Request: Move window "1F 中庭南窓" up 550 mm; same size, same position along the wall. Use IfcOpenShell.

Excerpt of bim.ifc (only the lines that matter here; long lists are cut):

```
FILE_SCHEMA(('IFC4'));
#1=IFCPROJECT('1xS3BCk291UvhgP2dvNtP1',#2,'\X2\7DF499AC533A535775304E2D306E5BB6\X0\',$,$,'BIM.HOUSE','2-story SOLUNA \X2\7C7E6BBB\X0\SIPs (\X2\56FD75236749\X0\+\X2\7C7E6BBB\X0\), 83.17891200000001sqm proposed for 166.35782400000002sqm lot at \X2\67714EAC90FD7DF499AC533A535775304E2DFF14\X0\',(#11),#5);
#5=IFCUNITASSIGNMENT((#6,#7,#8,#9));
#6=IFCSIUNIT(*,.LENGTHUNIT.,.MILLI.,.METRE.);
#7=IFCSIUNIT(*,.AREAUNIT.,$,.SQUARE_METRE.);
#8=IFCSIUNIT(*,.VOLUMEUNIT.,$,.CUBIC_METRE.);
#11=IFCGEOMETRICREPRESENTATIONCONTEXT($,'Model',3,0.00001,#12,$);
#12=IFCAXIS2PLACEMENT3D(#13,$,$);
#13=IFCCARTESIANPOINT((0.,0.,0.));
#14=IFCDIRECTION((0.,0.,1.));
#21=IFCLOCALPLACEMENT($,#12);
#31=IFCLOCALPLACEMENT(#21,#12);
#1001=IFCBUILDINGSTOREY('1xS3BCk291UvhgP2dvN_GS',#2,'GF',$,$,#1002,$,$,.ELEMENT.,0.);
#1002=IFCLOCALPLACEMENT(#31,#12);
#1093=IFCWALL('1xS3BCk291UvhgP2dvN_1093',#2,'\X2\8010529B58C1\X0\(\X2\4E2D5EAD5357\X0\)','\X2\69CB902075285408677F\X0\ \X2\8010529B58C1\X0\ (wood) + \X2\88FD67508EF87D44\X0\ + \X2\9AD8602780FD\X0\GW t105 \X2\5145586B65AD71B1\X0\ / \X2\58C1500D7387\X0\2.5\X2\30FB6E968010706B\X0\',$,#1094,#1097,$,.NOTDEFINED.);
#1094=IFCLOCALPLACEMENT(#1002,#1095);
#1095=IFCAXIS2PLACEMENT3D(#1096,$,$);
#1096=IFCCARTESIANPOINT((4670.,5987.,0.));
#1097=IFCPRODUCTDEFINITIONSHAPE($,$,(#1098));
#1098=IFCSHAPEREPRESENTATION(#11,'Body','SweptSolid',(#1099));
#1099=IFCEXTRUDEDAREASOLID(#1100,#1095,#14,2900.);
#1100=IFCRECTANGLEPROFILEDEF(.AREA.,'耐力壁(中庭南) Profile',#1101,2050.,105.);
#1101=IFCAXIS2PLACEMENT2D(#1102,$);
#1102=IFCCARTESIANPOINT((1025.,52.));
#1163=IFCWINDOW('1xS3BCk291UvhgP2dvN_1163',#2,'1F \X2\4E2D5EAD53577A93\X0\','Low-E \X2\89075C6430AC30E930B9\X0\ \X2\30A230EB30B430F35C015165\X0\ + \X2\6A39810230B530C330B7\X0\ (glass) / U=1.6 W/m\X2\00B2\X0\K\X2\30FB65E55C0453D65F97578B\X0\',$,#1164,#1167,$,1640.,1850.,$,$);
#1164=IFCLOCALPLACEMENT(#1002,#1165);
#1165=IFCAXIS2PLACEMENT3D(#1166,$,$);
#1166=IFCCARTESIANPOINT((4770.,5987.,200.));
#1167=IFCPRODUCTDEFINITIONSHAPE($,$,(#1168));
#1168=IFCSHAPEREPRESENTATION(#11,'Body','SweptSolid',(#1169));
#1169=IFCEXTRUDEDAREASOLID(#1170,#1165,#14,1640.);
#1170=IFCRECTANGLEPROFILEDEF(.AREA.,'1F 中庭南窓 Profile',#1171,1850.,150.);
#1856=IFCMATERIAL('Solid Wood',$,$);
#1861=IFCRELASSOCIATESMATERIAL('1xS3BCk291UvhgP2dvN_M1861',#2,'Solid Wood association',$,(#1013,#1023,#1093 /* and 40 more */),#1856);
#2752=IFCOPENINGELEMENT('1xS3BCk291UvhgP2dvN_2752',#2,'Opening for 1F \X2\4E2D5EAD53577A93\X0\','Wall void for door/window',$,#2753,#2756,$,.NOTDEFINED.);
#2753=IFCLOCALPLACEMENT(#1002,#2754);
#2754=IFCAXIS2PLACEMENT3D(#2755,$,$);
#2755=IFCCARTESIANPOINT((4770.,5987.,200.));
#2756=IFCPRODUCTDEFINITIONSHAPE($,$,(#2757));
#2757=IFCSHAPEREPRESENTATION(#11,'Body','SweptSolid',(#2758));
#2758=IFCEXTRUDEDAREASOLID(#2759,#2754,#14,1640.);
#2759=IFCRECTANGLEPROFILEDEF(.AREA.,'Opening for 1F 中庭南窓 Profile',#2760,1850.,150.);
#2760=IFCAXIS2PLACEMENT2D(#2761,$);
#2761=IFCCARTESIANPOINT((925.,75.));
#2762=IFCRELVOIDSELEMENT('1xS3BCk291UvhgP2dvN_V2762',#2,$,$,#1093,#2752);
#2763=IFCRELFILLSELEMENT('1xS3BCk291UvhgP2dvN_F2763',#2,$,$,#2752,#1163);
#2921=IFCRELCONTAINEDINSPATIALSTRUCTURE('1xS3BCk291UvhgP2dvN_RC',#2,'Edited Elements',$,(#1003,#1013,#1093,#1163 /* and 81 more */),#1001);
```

```python
import numpy as np
import ifcopenshell
import ifcopenshell.api.geometry
import ifcopenshell.util.placement
import ifcopenshell.util.unit

model = ifcopenshell.open("bim.ifc")
unit_scale = ifcopenshell.util.unit.calculate_unit_scale(model)

window = model.by_id(1163)
opening = window.FillsVoids[0].RelatingOpeningElement
dz = 550.0

shift = np.array([0.0, 0.0, dz])
# The window is not placed relative to its opening, so move both.
for product in (opening, window):
    matrix = ifcopenshell.util.placement.get_local_placement(product.ObjectPlacement)
    matrix[:3, 3] += shift
    ifcopenshell.api.geometry.edit_object_placement(model, product=product, matrix=matrix, is_si=False)

print(f"moved by {dz * unit_scale:+.3f} m")

model.write("bim_updated.ifc")
```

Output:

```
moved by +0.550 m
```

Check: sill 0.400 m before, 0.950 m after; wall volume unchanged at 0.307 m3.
